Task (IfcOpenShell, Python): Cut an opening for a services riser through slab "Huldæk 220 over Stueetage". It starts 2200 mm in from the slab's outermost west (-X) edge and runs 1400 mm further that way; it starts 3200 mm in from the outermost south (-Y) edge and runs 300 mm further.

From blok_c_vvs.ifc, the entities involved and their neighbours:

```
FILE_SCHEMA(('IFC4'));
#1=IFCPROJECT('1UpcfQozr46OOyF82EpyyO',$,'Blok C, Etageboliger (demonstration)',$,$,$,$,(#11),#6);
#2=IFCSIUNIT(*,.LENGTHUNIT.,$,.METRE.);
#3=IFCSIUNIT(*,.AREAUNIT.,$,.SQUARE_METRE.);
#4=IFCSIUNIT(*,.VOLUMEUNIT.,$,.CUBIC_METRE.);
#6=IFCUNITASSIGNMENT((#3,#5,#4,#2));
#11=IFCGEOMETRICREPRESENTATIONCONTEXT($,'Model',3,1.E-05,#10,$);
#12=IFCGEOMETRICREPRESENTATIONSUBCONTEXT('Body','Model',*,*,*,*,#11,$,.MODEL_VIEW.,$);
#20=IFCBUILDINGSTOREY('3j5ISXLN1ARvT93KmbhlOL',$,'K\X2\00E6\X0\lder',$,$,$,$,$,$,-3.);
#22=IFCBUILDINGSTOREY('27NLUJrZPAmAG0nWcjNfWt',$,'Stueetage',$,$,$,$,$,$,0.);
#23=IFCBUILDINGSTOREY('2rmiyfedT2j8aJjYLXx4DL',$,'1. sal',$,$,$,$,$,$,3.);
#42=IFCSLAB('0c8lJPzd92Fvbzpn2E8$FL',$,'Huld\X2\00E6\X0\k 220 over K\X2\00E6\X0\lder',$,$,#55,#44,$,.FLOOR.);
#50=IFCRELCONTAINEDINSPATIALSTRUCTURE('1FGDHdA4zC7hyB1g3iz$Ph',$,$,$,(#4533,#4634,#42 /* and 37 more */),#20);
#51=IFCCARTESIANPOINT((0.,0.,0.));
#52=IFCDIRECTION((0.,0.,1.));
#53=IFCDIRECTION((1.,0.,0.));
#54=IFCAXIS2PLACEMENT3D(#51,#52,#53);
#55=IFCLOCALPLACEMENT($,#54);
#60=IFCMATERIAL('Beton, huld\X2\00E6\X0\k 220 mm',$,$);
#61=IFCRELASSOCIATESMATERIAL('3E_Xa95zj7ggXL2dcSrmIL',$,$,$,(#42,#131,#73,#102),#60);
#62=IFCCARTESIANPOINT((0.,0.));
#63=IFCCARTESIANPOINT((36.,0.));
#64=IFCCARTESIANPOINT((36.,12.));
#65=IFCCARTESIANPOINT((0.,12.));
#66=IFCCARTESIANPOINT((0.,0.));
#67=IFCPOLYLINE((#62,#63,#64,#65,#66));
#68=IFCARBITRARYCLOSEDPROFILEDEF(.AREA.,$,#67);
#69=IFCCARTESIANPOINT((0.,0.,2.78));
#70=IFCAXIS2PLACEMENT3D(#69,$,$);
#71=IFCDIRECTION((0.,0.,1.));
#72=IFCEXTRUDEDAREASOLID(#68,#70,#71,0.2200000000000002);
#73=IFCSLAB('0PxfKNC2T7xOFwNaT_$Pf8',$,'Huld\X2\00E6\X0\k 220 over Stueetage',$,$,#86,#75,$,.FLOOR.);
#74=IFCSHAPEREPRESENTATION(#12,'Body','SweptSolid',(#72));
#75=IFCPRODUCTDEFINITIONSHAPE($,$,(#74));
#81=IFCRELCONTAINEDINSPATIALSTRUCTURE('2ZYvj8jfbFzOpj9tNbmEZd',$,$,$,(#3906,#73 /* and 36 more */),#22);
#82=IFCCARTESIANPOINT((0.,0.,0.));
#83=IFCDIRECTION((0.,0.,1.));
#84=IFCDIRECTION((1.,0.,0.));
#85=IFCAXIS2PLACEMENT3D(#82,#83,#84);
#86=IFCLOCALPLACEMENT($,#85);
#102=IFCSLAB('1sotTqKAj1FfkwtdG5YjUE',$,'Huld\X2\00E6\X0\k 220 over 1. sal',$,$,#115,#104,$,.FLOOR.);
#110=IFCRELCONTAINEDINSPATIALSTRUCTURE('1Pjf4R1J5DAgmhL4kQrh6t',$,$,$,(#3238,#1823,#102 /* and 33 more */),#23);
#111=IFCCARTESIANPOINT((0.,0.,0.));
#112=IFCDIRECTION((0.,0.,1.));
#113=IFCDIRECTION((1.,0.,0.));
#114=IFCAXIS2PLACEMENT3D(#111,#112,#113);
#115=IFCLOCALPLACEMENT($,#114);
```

```python
import numpy as np
import ifcopenshell
import ifcopenshell.api.feature
import ifcopenshell.api.geometry
import ifcopenshell.api.root
import ifcopenshell.geom
import ifcopenshell.util.placement
import ifcopenshell.util.representation
import ifcopenshell.util.shape
import ifcopenshell.util.unit

model = ifcopenshell.open("blok_c_vvs.ifc")
unit_scale = ifcopenshell.util.unit.calculate_unit_scale(model)
settings = ifcopenshell.geom.settings()


def volume(element):
    """Net volume in cubic metres, openings subtracted."""
    shape = ifcopenshell.geom.create_shape(settings, element)
    return ifcopenshell.util.shape.get_volume(shape.geometry)


slab = model.by_guid("0PxfKNC2T7xOFwNaT_$Pf8")
before = volume(slab)

# Extent in the slab's own axes, in metres. The edges named are its -X and -Y sides.
slab_shape = ifcopenshell.geom.create_shape(settings, slab)
vertices = ifcopenshell.util.shape.get_vertices(slab_shape.geometry)
x_min, y_min, bottom = vertices.min(axis=0)
top = vertices[:, 2].max()

opening = ifcopenshell.api.root.create_entity(model, ifc_class="IfcOpeningElement", name="Services riser opening", predefined_type="OPENING")
context = ifcopenshell.util.representation.get_context(model, "Model", "Body", "MODEL_VIEW")
width, depth = 1.4, 0.3
outline = [(0.0, 0.0), (width, 0.0), (width, depth), (0.0, depth), (0.0, 0.0)]
# Overshoot both faces by 50 mm so the cut is clean.
shape = ifcopenshell.api.geometry.add_slab_representation(
    model, context=context, depth=top - bottom + 0.1, polyline=outline
)
ifcopenshell.api.geometry.assign_representation(model, product=opening, representation=shape)

matrix = ifcopenshell.util.placement.get_local_placement(slab.ObjectPlacement)
matrix[:, 3] = matrix @ np.append(np.array([x_min + 2.2, y_min + 3.2, bottom - 0.05]) / unit_scale, 1.0)
ifcopenshell.api.geometry.edit_object_placement(model, product=opening, matrix=matrix, is_si=False)
ifcopenshell.api.feature.add_feature(model, feature=opening, element=slab)

after = volume(slab)

print(f"slab volume {before:.3f} -> {after:.3f} m3")

model.write("blok_c_vvs_updated.ifc")
```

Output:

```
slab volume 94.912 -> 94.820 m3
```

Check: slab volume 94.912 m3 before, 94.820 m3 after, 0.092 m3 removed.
